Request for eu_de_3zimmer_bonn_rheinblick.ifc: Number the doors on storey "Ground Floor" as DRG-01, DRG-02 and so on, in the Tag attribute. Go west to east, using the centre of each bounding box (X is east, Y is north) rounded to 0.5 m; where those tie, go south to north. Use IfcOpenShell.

First a look at what the model holds.

```python
import ifcopenshell
import ifcopenshell.util.element
import ifcopenshell.util.placement

model = ifcopenshell.open("eu_de_3zimmer_bonn_rheinblick.ifc")
print(model.schema)
storey = next(s for s in model.by_type("IfcBuildingStorey") if s.Name == "Ground Floor")
doors = [e for e in ifcopenshell.util.element.get_decomposition(storey) if e.is_a("IfcDoor")]
for e in sorted(doors, key=lambda e: e.id()):
    origin = ifcopenshell.util.placement.get_local_placement(e.ObjectPlacement)[:3, 3]
    print(e.id(), e.Tag, e.Name, origin.round(2) + 0.0, sep=" | ")
```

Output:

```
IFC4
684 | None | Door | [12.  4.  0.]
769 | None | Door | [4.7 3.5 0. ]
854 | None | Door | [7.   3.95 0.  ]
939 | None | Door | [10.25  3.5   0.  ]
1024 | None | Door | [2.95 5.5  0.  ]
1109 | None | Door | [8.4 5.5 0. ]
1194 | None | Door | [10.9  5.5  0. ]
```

```python
import ifcopenshell
import ifcopenshell.geom
import ifcopenshell.util.element
import ifcopenshell.util.shape

model = ifcopenshell.open("eu_de_3zimmer_bonn_rheinblick.ifc")
settings = ifcopenshell.geom.settings()
settings.set("use-world-coords", True)


def centre(element):
    shape = ifcopenshell.geom.create_shape(settings, element)
    return ifcopenshell.util.shape.get_bbox_centroid(shape.geometry)


storey = next(s for s in model.by_type("IfcBuildingStorey") if s.Name == "Ground Floor")
doors = [e for e in ifcopenshell.util.element.get_decomposition(storey) if e.is_a("IfcDoor")]

# Insertion points can sit at a corner or the storey origin, so sort by the geometry (in metres).
centres = {e: centre(e) for e in doors}
doors.sort(key=lambda e: (round(centres[e][0] / 0.5), centres[e][1]))

for i, e in enumerate(doors, start=1):
    number = f"DRG-{i:02d}"
    e.Tag = number
    print(e.id(), number)

model.write("eu_de_3zimmer_bonn_rheinblick_v2.ifc")
```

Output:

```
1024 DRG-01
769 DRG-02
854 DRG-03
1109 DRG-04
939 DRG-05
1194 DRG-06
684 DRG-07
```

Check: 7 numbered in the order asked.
